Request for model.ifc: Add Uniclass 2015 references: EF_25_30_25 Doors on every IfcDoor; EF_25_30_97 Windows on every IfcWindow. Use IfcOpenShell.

First a look at what the model holds.

```python
import ifcopenshell

model = ifcopenshell.open("model.ifc")
print(model.schema)
print("classifications:", [c.Name for c in model.by_type("IfcClassification")])
for ifc_class in ("IfcDoor", "IfcRoof", "IfcStair", "IfcWall", "IfcWindow"):
    print(ifc_class, len(model.by_type(ifc_class)))
```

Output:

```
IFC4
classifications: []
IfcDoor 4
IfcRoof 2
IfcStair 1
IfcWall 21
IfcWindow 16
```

```python
import ifcopenshell
import ifcopenshell.api.classification

model = ifcopenshell.open("model.ifc")

system = ifcopenshell.api.classification.add_classification(model, classification="Uniclass 2015")

codes = {
    "IfcDoor": ("EF_25_30_25", "Doors"),
    "IfcWindow": ("EF_25_30_97", "Windows"),
}
for ifc_class, (code, name) in codes.items():
    products = model.by_type(ifc_class)
    ifcopenshell.api.classification.add_reference(
        model, products=products, classification=system, identification=code, name=name
    )
    print(code, len(products))

model.write("model_v2.ifc")
```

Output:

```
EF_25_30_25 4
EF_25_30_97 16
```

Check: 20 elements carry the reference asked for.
